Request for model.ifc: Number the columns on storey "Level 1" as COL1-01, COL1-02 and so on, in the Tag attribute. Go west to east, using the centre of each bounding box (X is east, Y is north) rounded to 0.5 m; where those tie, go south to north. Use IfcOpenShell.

First a look at what the model holds.

```python
import ifcopenshell
import ifcopenshell.util.element
import ifcopenshell.util.placement

model = ifcopenshell.open("model.ifc")
print(model.schema)
storey = next(s for s in model.by_type("IfcBuildingStorey") if s.Name == "Level 1")
columns = [e for e in ifcopenshell.util.element.get_decomposition(storey) if e.is_a("IfcColumn")]
for e in sorted(columns, key=lambda e: e.id()):
    origin = ifcopenshell.util.placement.get_local_placement(e.ObjectPlacement)[:3, 3]
    print(e.id(), e.Tag, e.Name, origin.round(2) + 0.0, sep=" | ")
```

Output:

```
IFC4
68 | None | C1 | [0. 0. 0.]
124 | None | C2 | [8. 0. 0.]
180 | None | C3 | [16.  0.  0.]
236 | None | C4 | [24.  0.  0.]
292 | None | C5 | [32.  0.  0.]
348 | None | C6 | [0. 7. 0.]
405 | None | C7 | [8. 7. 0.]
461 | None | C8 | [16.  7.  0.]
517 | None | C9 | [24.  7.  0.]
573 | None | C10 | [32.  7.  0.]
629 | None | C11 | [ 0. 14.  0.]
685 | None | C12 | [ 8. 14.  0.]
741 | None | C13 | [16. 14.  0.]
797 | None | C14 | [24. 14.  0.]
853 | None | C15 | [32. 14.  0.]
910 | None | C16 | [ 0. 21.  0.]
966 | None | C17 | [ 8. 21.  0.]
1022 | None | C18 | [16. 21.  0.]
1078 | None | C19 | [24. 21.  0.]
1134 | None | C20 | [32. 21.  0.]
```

```python
import ifcopenshell
import ifcopenshell.geom
import ifcopenshell.util.element
import ifcopenshell.util.shape

model = ifcopenshell.open("model.ifc")
settings = ifcopenshell.geom.settings()
settings.set("use-world-coords", True)


def centre(element):
    shape = ifcopenshell.geom.create_shape(settings, element)
    return ifcopenshell.util.shape.get_bbox_centroid(shape.geometry)


storey = next(s for s in model.by_type("IfcBuildingStorey") if s.Name == "Level 1")
columns = [e for e in ifcopenshell.util.element.get_decomposition(storey) if e.is_a("IfcColumn")]

# Insertion points can sit at a corner or the storey origin, so sort by the geometry (in metres).
centres = {e: centre(e) for e in columns}
columns.sort(key=lambda e: (round(centres[e][0] / 0.5), centres[e][1]))

for i, e in enumerate(columns, start=1):
    number = f"COL1-{i:02d}"
    e.Tag = number
    print(e.id(), number)

model.write("model_updated.ifc")
```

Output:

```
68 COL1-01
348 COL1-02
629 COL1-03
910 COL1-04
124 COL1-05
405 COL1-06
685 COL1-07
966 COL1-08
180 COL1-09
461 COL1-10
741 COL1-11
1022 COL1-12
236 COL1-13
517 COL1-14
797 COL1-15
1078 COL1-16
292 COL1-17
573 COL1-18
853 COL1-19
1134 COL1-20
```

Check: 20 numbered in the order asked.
